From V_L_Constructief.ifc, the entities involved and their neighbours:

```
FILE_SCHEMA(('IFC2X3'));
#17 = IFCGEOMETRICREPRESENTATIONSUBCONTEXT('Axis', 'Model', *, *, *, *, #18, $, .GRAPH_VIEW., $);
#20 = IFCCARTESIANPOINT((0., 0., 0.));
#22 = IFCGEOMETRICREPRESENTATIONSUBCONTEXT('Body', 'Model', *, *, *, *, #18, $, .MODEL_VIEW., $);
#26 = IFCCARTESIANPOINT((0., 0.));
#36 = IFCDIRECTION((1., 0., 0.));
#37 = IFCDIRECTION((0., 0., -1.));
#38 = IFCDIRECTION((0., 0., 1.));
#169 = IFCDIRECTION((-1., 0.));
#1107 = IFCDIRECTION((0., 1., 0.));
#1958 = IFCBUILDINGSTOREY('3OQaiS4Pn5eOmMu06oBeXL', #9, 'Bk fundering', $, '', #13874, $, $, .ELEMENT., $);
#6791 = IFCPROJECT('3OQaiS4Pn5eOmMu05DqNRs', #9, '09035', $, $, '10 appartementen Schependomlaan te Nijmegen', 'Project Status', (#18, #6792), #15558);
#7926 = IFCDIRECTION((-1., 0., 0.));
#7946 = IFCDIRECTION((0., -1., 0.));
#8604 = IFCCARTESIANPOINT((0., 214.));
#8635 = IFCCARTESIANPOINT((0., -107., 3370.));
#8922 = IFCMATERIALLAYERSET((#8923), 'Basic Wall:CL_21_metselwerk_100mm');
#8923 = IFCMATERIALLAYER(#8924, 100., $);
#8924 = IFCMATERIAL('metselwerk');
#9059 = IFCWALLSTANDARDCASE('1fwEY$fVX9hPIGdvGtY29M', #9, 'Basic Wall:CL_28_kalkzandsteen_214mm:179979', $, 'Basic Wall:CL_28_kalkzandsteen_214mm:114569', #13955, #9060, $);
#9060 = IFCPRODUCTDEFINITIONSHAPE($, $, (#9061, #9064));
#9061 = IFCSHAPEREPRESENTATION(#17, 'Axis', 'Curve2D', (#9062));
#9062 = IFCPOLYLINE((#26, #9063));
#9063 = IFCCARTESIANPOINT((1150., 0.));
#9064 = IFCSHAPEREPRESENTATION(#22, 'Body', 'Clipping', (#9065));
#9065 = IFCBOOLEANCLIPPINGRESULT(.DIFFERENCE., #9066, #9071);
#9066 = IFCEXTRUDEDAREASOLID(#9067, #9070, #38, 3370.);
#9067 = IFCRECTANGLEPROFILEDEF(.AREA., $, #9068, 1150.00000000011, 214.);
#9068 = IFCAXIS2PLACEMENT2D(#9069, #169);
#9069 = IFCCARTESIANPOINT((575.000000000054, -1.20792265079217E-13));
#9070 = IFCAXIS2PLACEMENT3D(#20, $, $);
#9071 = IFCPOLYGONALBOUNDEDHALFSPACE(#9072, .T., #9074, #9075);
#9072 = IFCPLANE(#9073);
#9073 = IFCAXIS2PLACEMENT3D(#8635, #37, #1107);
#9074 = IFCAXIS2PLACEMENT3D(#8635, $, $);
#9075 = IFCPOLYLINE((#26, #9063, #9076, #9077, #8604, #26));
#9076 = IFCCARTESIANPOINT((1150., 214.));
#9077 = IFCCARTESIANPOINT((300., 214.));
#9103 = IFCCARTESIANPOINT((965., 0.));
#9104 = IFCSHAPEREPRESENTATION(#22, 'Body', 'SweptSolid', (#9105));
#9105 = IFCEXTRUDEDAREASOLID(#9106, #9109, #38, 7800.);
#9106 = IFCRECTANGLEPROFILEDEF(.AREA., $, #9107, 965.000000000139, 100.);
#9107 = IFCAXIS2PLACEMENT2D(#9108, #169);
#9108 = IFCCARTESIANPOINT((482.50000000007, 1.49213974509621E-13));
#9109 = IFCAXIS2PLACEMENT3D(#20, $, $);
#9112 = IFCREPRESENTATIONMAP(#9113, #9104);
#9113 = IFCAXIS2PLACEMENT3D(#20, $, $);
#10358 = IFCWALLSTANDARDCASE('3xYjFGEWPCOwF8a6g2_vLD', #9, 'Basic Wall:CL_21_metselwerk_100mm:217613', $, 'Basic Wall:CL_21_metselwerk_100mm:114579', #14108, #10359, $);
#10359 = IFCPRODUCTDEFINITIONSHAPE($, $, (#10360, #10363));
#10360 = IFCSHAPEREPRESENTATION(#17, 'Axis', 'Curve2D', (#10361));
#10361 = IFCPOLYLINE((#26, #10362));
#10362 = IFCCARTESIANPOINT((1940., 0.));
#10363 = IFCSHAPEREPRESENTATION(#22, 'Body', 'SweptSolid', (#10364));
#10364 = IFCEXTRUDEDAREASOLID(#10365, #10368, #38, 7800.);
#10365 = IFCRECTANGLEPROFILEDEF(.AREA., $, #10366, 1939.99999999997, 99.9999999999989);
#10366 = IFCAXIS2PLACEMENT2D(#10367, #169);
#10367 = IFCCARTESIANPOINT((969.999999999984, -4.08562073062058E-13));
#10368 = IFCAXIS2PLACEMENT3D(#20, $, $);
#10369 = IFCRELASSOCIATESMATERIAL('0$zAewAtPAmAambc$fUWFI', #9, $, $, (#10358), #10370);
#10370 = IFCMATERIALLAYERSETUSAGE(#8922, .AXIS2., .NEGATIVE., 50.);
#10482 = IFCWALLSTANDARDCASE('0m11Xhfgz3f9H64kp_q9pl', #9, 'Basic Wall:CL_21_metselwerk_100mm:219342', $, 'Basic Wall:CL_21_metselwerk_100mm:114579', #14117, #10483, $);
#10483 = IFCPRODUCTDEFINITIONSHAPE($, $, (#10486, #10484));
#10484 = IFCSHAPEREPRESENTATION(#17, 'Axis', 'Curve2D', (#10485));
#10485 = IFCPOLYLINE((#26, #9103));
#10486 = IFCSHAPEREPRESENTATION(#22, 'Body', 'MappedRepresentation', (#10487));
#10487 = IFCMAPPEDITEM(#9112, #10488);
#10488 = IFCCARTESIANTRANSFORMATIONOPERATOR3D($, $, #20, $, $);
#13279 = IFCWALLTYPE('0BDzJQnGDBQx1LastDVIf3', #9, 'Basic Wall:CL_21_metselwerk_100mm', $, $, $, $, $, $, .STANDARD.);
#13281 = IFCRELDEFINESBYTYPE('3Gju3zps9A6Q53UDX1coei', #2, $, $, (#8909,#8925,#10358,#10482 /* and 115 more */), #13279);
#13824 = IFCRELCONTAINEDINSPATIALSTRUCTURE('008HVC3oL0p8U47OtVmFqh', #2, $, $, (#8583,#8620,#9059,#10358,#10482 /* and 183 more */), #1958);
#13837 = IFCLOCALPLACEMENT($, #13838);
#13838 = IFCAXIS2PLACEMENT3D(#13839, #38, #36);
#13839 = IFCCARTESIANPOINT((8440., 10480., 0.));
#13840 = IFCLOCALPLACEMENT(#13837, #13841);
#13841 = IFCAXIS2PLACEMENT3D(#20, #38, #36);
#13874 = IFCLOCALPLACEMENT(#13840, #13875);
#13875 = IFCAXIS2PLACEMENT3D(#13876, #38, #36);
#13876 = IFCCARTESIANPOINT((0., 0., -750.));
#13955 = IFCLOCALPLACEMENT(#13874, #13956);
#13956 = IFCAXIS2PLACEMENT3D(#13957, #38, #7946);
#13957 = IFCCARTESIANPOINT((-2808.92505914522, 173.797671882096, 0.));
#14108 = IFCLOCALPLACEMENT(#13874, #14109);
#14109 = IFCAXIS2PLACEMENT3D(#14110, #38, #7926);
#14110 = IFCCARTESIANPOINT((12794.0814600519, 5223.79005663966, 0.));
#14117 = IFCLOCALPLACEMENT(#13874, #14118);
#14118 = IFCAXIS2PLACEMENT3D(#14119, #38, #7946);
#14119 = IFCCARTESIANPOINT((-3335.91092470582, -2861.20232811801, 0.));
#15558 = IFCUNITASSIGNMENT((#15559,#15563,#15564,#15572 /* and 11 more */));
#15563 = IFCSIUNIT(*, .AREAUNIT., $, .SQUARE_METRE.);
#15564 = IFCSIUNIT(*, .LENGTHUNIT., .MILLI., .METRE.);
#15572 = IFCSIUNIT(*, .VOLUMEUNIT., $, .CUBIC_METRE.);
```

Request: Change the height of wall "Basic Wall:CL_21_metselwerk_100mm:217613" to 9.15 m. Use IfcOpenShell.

```python
import ifcopenshell
import ifcopenshell.geom
import ifcopenshell.util.representation
import ifcopenshell.util.shape
import ifcopenshell.util.unit

model = ifcopenshell.open("V_L_Constructief.ifc")
unit_scale = ifcopenshell.util.unit.calculate_unit_scale(model)
settings = ifcopenshell.geom.settings()


def volume(element):
    """Net volume in cubic metres, openings subtracted."""
    shape = ifcopenshell.geom.create_shape(settings, element)
    return ifcopenshell.util.shape.get_volume(shape.geometry)


wall = model.by_guid("3xYjFGEWPCOwF8a6g2_vLD")
before = volume(wall)

body = ifcopenshell.util.representation.get_representation(wall, "Model", "Body")
solid = body.Items[0]
old_height = solid.Depth
solid.Depth = 9.15 / unit_scale
after = volume(wall)

print(f"height {old_height:g} -> {solid.Depth:g}, volume {before:.3f} -> {after:.3f} m3")

model.write("V_L_Constructief_v2.ifc")
```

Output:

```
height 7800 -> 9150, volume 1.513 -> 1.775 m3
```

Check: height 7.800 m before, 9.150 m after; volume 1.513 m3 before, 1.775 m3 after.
